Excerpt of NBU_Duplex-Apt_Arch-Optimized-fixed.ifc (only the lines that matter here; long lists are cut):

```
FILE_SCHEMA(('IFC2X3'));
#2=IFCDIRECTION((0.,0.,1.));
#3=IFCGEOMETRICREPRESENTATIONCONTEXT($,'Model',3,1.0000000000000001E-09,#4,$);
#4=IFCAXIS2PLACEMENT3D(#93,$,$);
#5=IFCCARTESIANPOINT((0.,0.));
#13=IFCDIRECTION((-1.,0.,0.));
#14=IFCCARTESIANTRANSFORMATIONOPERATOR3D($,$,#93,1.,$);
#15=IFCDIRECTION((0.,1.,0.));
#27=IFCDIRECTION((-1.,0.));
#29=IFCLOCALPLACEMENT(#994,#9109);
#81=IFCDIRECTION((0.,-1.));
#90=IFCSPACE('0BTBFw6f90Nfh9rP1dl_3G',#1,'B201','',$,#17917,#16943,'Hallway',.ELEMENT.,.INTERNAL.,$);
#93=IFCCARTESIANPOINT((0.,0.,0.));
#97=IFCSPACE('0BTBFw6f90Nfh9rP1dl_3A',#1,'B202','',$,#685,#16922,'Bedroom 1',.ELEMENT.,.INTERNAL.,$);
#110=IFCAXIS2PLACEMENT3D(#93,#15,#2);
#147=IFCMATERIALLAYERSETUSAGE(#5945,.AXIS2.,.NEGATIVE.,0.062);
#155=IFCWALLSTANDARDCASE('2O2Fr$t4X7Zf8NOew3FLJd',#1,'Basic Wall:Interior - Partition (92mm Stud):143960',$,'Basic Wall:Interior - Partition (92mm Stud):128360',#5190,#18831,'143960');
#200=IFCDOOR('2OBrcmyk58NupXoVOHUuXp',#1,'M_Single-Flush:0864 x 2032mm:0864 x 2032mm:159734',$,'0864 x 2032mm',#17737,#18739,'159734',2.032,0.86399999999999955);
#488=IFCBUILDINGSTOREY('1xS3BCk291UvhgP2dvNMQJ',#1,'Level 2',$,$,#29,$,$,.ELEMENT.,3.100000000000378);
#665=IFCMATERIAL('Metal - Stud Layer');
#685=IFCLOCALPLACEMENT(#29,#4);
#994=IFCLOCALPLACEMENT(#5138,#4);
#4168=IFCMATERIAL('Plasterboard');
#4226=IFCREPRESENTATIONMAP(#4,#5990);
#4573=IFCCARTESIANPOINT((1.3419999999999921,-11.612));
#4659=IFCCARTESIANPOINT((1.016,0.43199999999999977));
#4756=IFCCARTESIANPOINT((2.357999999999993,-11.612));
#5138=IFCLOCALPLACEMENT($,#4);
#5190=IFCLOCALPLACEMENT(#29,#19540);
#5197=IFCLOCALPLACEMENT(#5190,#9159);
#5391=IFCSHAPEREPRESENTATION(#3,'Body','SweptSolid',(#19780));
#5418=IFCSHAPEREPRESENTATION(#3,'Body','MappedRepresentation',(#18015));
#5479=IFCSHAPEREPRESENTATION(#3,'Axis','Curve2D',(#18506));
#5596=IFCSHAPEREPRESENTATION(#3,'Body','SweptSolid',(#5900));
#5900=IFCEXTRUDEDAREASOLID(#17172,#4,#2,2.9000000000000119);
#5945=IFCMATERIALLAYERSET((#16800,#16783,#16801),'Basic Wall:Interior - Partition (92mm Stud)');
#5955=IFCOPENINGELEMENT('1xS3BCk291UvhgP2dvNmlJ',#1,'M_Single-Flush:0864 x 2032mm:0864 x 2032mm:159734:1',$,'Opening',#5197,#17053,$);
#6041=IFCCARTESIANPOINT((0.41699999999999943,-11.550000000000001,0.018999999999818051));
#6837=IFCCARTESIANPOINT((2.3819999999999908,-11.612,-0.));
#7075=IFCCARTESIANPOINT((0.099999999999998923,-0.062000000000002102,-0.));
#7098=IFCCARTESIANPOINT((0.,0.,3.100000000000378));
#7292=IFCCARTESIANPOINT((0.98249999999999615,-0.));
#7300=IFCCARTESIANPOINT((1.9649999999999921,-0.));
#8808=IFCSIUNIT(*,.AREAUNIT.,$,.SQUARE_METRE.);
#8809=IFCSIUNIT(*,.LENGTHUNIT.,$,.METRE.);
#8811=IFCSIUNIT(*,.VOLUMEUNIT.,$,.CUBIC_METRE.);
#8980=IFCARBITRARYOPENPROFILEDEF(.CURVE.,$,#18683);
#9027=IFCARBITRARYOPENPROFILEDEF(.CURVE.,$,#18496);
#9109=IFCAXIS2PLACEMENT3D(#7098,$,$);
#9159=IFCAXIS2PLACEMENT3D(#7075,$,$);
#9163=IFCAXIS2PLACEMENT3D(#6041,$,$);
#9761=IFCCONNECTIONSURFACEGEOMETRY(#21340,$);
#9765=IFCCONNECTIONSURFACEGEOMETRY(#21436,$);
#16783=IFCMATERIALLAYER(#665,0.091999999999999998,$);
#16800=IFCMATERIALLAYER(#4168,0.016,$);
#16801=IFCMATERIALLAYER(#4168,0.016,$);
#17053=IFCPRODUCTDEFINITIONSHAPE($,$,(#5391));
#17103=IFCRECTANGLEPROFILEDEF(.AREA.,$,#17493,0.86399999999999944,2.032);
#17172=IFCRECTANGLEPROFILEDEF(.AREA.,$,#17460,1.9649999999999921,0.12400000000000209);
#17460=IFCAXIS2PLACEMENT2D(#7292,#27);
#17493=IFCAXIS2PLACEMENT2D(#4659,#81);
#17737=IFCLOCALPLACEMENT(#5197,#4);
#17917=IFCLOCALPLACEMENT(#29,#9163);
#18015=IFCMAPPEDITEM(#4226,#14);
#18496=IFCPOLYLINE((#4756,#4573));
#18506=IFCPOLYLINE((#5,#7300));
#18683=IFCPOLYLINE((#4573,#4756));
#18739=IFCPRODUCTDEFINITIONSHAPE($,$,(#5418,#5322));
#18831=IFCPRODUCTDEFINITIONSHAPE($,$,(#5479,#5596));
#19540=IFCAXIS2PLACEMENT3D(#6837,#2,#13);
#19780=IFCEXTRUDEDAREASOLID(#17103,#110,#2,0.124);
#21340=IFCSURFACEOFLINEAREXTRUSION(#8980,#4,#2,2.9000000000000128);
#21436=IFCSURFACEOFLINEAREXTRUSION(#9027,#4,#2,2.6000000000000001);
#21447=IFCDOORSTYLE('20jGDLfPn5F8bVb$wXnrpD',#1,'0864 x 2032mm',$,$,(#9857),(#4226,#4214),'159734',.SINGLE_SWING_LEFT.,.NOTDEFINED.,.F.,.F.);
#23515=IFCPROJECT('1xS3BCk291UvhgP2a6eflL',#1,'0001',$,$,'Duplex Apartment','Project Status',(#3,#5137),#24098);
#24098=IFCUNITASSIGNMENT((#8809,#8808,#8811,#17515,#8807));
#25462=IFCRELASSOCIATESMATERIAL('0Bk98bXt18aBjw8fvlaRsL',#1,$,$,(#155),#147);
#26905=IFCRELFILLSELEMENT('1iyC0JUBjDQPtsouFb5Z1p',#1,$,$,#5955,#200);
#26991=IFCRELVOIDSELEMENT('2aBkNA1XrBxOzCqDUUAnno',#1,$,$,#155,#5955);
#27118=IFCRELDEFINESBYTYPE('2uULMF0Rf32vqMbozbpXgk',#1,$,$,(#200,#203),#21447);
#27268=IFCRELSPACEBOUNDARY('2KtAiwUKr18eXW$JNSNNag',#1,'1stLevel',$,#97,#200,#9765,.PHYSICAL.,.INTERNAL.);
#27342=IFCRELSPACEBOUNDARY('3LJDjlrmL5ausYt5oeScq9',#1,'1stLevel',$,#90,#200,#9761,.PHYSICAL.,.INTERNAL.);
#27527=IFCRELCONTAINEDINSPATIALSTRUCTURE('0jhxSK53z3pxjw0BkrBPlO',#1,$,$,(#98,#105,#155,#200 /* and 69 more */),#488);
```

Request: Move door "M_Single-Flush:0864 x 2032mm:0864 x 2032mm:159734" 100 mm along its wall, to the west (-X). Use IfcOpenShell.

```python
import numpy as np
import ifcopenshell
import ifcopenshell.api.geometry
import ifcopenshell.util.placement
import ifcopenshell.util.unit

model = ifcopenshell.open("NBU_Duplex-Apt_Arch-Optimized-fixed.ifc")
unit_scale = ifcopenshell.util.unit.calculate_unit_scale(model)

door = model.by_guid("2OBrcmyk58NupXoVOHUuXp")
opening = door.FillsVoids[0].RelatingOpeningElement
wall = opening.VoidsElements[0].RelatingBuildingElement

wall_matrix = ifcopenshell.util.placement.get_local_placement(wall.ObjectPlacement)
shift = wall_matrix[:3, 0] * 0.1 / unit_scale
before = ifcopenshell.util.placement.get_local_placement(door.ObjectPlacement)[:3, 3].copy()

# The door is placed relative to its opening, so it follows when the opening moves.
matrix = ifcopenshell.util.placement.get_local_placement(opening.ObjectPlacement)
matrix[:3, 3] += shift
ifcopenshell.api.geometry.edit_object_placement(
    model, product=opening, matrix=matrix, is_si=False, should_transform_children=True
)

# Space boundary surfaces are stored in each space's coordinates; move them too.
for rel in door.ProvidesBoundaries:
    if not rel.ConnectionGeometry:
        continue
    surface = rel.ConnectionGeometry.SurfaceOnRelatingElement
    space_matrix = ifcopenshell.util.placement.get_local_placement(rel.RelatingSpace.ObjectPlacement)
    point = np.array(surface.Position.Location.Coordinates) + space_matrix[:3, :3].T @ shift
    surface.Position = model.createIfcAxis2Placement3D(
        model.createIfcCartesianPoint(point.tolist()), surface.Position.Axis, surface.Position.RefDirection
    )

after = ifcopenshell.util.placement.get_local_placement(door.ObjectPlacement)[:3, 3]
print("door moved by", (after - before).round(3) + 0.0)

model.write("NBU_Duplex-Apt_Arch-Optimized-fixed_rev.ifc")
```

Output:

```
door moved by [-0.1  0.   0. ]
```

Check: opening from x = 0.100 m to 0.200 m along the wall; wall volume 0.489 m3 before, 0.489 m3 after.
